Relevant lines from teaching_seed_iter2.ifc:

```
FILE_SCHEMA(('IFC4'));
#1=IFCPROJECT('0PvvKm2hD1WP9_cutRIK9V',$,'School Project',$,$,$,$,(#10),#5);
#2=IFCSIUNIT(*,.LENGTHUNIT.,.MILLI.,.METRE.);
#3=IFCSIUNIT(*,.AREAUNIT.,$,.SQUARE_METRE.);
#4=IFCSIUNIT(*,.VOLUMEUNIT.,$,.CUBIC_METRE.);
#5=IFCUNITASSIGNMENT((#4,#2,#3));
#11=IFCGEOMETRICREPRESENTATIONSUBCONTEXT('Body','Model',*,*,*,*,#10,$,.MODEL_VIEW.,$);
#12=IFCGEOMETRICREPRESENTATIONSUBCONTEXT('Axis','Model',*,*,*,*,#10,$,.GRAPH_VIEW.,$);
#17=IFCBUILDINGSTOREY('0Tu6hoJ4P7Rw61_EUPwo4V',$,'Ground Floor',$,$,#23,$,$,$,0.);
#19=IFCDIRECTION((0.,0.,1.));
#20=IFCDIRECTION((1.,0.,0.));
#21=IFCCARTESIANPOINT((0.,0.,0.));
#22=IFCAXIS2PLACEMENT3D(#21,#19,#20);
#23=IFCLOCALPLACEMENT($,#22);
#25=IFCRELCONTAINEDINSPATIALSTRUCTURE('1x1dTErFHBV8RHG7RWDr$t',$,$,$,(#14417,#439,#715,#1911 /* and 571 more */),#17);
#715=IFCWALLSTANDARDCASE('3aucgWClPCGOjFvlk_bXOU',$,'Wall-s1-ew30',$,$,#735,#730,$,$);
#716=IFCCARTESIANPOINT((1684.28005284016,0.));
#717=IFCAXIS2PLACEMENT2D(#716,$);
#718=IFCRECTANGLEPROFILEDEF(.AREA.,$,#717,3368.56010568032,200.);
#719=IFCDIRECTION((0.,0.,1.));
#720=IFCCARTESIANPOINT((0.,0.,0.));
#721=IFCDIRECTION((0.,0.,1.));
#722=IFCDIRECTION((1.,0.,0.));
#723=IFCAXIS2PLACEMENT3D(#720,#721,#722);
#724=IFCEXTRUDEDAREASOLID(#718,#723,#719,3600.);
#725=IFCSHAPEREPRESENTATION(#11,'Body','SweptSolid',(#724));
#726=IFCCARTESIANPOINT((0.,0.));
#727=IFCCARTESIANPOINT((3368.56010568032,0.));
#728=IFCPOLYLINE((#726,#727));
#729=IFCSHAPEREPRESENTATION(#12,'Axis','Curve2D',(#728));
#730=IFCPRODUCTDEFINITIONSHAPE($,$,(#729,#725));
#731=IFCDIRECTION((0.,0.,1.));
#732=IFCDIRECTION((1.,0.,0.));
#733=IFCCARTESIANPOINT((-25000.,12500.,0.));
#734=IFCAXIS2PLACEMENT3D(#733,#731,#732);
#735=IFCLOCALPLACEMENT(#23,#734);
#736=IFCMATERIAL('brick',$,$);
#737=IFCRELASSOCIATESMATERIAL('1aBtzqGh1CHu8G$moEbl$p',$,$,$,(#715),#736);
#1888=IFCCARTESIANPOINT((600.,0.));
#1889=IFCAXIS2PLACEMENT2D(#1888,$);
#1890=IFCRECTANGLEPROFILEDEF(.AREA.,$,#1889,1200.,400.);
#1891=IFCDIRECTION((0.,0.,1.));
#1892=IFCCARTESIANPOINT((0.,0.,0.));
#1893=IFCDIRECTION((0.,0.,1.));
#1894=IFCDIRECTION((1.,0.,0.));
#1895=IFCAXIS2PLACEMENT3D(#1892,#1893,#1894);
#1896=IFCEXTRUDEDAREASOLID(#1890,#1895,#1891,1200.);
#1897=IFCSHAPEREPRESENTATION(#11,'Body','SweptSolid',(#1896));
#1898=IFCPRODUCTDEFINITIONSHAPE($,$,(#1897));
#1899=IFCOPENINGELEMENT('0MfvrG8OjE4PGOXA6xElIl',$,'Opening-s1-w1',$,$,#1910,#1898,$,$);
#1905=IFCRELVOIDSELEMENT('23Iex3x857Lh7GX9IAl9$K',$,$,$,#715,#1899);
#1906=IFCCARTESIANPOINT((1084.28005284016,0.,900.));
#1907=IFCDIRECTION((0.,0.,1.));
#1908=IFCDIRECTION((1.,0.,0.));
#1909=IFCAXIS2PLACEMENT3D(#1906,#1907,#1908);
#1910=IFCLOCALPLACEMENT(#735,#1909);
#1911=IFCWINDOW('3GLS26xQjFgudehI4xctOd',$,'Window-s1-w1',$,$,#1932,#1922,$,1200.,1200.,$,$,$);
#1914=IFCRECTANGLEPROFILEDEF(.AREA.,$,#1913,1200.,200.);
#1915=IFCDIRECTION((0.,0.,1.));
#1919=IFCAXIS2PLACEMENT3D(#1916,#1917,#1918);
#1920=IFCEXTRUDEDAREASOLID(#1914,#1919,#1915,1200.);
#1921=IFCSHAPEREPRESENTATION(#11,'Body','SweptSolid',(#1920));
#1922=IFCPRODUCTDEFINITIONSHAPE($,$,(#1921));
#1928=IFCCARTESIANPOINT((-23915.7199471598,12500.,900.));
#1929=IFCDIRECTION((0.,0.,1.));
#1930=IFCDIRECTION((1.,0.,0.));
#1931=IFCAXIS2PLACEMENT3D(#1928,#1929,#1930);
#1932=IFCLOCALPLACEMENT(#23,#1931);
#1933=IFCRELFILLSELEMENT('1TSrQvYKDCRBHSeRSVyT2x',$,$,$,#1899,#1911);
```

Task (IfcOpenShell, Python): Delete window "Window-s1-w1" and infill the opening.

```python
import ifcopenshell
import ifcopenshell.api.feature
import ifcopenshell.api.root
import ifcopenshell.geom
import ifcopenshell.util.shape

model = ifcopenshell.open("teaching_seed_iter2.ifc")
settings = ifcopenshell.geom.settings()


def volume(element):
    """Net volume in cubic metres, openings subtracted."""
    shape = ifcopenshell.geom.create_shape(settings, element)
    return ifcopenshell.util.shape.get_volume(shape.geometry)


window = model.by_guid("3GLS26xQjFgudehI4xctOd")
opening = window.FillsVoids[0].RelatingOpeningElement
wall = opening.VoidsElements[0].RelatingBuildingElement
before = volume(wall)

ifcopenshell.api.root.remove_product(model, product=window)
ifcopenshell.api.feature.remove_feature(model, feature=opening)

after = volume(wall)

print(f"wall volume {before:.3f} -> {after:.3f} m3")

model.write("teaching_seed_iter2_edited.ifc")
```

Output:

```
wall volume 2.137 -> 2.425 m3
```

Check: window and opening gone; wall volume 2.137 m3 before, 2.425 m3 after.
